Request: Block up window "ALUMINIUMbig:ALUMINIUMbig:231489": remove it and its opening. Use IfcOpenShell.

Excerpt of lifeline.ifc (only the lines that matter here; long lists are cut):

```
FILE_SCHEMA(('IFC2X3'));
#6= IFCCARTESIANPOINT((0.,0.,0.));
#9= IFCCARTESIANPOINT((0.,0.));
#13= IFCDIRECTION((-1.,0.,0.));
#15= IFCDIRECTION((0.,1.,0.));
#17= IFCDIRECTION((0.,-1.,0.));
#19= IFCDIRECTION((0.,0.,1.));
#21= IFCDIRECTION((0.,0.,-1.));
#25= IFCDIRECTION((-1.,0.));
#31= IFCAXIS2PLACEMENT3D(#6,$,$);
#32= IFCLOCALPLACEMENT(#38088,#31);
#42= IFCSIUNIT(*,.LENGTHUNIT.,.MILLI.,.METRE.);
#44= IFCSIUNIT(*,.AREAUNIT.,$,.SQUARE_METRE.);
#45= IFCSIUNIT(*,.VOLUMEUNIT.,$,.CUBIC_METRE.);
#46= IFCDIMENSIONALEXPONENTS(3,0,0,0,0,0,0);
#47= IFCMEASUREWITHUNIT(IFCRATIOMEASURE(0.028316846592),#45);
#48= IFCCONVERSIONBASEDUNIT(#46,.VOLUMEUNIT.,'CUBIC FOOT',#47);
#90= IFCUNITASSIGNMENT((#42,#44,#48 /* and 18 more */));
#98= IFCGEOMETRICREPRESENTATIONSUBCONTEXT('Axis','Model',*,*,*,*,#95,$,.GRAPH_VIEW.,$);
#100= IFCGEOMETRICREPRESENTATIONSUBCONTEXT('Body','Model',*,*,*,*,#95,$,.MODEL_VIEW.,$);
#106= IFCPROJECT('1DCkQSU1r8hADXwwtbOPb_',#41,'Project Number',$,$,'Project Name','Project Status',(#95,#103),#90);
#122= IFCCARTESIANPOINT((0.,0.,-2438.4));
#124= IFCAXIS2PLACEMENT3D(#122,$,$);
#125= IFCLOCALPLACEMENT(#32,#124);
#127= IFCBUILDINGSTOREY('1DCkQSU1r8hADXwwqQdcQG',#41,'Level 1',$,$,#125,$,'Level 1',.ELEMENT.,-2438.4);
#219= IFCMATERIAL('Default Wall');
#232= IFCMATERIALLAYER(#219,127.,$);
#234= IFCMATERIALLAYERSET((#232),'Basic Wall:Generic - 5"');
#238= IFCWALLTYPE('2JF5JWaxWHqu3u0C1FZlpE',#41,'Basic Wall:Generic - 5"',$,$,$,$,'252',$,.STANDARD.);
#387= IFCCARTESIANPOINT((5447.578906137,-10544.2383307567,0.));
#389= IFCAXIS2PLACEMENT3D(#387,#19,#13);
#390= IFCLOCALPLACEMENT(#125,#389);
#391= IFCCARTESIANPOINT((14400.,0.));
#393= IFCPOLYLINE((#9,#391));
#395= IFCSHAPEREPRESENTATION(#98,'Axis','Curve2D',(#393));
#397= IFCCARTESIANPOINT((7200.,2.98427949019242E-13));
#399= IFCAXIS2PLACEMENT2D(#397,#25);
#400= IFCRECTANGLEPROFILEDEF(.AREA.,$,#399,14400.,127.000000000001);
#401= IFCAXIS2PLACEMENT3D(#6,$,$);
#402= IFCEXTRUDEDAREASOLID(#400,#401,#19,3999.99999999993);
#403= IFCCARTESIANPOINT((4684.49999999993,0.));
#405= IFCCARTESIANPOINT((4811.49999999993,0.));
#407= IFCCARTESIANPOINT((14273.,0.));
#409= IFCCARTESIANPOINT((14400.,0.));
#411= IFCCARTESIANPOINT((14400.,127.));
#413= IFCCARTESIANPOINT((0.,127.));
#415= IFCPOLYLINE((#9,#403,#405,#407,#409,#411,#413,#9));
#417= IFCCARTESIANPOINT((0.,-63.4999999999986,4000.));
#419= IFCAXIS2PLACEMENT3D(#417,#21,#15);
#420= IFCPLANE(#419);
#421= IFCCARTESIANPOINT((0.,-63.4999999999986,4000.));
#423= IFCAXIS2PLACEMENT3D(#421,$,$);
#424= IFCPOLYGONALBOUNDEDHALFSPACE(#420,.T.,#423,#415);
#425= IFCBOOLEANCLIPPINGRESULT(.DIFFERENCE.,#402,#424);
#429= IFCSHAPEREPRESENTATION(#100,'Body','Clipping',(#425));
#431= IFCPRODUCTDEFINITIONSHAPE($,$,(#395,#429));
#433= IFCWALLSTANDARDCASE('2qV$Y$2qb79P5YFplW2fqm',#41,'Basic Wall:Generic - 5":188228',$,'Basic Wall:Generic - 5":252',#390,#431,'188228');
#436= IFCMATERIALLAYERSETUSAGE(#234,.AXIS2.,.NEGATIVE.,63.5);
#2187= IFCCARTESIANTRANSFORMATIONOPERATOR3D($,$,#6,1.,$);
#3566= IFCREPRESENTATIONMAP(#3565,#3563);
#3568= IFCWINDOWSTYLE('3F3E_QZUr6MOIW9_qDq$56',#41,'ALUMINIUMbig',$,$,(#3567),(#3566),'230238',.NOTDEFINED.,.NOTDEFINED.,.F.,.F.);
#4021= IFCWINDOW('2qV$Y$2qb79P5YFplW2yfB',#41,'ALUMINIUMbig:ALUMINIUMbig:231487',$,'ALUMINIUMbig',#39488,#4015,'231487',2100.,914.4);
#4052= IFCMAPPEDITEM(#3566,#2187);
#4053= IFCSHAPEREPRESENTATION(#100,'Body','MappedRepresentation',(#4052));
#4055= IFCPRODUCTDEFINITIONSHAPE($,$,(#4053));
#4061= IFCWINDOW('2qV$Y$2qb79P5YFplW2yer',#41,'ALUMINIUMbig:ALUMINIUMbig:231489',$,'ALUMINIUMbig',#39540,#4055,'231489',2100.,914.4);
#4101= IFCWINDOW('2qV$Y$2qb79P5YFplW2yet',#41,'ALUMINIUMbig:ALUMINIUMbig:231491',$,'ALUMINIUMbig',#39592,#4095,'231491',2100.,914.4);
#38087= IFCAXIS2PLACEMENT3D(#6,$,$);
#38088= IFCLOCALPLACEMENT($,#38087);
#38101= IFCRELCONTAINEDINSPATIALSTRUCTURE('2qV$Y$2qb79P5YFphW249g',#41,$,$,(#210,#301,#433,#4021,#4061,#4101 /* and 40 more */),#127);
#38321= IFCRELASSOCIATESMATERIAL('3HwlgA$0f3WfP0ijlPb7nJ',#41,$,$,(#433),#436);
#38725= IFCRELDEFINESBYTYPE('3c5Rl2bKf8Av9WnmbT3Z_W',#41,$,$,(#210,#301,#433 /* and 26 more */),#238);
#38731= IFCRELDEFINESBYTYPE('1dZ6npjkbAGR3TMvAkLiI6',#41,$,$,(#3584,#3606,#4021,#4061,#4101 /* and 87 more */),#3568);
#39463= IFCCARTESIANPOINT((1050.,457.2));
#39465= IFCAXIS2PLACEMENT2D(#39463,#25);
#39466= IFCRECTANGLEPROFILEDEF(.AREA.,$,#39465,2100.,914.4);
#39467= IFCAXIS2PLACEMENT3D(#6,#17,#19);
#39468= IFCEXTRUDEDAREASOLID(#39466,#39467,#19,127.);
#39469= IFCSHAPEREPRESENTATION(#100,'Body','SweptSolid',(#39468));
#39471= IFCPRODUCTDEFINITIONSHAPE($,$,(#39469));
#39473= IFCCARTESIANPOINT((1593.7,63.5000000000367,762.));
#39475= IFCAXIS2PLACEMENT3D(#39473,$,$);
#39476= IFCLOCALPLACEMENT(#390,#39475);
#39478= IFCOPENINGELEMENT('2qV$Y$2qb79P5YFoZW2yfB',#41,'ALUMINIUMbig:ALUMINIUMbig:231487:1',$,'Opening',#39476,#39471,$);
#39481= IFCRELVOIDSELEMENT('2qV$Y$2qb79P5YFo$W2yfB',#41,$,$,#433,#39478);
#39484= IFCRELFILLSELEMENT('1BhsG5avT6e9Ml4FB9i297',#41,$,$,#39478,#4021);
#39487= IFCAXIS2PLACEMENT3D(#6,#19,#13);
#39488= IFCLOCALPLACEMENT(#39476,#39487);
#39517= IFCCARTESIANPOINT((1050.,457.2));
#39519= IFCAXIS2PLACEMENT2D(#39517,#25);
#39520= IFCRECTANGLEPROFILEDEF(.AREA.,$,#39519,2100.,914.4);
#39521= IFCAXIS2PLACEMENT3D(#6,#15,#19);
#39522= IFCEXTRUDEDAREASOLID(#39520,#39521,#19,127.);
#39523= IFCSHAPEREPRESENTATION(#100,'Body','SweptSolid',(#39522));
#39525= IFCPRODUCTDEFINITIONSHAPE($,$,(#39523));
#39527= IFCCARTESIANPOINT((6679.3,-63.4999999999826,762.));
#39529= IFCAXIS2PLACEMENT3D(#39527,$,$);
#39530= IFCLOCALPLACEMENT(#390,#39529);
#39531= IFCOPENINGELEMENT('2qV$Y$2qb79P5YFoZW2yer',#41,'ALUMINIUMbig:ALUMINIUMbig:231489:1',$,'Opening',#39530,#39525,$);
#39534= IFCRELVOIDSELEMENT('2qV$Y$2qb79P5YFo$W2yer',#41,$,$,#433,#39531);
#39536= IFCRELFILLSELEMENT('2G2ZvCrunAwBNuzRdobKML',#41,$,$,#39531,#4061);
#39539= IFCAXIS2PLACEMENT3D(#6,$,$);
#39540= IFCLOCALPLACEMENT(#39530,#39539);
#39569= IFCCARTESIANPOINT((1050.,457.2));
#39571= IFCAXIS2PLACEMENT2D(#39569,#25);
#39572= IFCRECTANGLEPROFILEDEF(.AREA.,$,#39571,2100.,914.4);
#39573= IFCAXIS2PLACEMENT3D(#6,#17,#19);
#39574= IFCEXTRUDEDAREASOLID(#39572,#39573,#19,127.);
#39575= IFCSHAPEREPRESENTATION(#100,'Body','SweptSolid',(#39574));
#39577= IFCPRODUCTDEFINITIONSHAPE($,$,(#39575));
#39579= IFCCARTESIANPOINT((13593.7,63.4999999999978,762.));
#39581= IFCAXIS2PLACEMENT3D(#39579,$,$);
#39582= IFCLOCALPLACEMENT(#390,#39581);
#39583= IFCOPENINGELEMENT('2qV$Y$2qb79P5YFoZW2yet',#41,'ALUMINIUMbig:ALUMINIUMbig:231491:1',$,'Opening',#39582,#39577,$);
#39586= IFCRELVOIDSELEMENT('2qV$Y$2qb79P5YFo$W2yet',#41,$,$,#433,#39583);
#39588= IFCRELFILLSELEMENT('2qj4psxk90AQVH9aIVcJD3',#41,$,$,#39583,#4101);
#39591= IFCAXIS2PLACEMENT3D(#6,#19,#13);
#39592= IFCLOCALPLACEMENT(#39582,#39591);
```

```python
import ifcopenshell
import ifcopenshell.api.feature
import ifcopenshell.api.root
import ifcopenshell.geom
import ifcopenshell.util.shape

model = ifcopenshell.open("lifeline.ifc")
settings = ifcopenshell.geom.settings()


def volume(element):
    """Net volume in cubic metres, openings subtracted."""
    shape = ifcopenshell.geom.create_shape(settings, element)
    return ifcopenshell.util.shape.get_volume(shape.geometry)


window = model.by_guid("2qV$Y$2qb79P5YFplW2yer")
opening = window.FillsVoids[0].RelatingOpeningElement
wall = opening.VoidsElements[0].RelatingBuildingElement
before = volume(wall)

ifcopenshell.api.root.remove_product(model, product=window)
ifcopenshell.api.feature.remove_feature(model, feature=opening)

after = volume(wall)

print(f"wall volume {before:.3f} -> {after:.3f} m3")

model.write("lifeline_rev.ifc")
```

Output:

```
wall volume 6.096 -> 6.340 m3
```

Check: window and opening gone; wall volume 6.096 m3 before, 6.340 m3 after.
